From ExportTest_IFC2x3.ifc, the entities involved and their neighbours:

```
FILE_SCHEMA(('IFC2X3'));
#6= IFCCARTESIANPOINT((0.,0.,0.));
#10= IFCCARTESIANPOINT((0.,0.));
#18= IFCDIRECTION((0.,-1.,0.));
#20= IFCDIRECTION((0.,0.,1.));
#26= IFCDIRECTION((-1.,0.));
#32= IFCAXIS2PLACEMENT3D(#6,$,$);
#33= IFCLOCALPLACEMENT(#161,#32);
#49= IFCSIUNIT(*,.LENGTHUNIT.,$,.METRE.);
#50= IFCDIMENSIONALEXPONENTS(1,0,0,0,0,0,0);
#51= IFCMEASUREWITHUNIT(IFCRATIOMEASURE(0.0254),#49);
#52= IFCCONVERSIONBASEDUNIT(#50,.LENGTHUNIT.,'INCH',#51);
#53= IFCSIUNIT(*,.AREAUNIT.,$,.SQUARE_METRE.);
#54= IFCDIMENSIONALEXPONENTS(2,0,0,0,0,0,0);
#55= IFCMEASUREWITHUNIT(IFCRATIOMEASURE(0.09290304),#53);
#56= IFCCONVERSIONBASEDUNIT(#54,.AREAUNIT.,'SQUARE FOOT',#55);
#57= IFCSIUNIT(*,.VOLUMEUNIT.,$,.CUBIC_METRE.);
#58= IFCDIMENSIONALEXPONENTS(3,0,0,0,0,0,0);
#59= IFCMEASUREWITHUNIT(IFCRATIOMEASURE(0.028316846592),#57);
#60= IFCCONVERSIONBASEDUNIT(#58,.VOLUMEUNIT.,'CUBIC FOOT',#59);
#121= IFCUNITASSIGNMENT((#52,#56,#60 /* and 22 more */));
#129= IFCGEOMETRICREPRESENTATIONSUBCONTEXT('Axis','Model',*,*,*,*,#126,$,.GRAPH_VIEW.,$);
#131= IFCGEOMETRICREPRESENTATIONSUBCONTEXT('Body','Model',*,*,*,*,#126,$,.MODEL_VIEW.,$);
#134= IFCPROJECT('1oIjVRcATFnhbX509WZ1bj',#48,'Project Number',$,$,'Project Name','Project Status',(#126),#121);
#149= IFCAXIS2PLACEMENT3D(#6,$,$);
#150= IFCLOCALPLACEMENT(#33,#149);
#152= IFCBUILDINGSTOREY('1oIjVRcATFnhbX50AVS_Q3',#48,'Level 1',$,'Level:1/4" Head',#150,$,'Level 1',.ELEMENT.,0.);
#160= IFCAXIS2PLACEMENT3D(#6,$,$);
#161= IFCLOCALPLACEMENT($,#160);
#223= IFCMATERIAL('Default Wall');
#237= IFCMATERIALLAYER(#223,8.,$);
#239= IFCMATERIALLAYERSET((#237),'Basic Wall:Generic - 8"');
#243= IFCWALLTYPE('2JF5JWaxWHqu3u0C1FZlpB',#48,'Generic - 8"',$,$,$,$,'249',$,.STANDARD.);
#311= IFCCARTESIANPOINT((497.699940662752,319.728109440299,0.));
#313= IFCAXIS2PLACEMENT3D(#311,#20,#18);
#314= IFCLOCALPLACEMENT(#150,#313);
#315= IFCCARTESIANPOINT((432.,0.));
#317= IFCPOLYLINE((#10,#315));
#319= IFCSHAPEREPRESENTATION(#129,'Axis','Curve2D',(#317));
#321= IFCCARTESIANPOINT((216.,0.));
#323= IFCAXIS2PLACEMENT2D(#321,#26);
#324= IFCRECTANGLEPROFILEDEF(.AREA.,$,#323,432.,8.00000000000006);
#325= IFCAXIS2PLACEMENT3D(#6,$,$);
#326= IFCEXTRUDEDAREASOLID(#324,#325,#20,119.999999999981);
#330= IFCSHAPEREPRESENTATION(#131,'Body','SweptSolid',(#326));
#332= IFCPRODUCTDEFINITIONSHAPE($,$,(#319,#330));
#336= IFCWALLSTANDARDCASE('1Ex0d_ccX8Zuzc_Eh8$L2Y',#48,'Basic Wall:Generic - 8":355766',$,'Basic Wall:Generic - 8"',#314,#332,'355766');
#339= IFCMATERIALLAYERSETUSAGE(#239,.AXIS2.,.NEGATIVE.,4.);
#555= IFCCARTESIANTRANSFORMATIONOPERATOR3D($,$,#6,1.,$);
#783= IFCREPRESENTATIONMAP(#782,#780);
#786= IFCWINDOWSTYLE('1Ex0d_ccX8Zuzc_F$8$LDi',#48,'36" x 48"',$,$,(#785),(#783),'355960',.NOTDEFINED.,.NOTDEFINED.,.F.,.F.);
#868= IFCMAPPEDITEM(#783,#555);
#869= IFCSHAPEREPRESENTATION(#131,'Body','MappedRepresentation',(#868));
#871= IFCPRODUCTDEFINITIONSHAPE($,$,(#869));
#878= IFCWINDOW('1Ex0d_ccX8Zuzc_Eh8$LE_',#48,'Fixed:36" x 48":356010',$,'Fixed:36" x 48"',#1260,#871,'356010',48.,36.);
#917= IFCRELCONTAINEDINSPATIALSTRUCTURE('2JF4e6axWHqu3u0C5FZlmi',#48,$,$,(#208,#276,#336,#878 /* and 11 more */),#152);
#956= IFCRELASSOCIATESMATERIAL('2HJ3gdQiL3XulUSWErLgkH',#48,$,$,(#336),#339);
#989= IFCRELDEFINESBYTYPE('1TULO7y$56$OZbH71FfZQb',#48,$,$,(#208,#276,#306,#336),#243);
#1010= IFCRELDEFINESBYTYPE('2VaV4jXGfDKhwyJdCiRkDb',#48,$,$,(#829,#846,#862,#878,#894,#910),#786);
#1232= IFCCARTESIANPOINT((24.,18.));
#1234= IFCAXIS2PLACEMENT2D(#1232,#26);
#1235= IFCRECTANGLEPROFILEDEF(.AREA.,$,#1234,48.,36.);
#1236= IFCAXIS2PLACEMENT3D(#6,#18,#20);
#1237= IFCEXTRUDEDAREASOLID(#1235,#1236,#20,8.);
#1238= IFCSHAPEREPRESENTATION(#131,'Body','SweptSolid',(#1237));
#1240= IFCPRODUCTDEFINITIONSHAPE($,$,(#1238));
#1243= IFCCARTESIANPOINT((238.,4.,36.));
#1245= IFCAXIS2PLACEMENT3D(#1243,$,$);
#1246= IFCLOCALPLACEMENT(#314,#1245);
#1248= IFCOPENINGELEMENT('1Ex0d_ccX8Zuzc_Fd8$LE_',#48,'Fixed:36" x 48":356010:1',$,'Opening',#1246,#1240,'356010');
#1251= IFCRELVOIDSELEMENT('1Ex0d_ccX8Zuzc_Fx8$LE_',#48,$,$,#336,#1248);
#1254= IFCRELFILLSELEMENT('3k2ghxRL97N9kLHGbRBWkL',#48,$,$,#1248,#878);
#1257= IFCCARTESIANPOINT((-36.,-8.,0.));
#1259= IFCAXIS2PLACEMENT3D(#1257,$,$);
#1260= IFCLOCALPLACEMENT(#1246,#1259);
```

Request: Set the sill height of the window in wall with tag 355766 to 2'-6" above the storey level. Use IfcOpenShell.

```python
import numpy as np
import ifcopenshell
import ifcopenshell.api.geometry
import ifcopenshell.geom
import ifcopenshell.util.element
import ifcopenshell.util.placement
import ifcopenshell.util.shape
import ifcopenshell.util.unit

model = ifcopenshell.open("ExportTest_IFC2x3.ifc")
unit_scale = ifcopenshell.util.unit.calculate_unit_scale(model)

window = model.by_guid("1Ex0d_ccX8Zuzc_Eh8$LE_")
opening = window.FillsVoids[0].RelatingOpeningElement
storey = ifcopenshell.util.element.get_container(window, ifc_class="IfcBuildingStorey")
level = ifcopenshell.util.placement.get_local_placement(storey.ObjectPlacement)[2, 3]

# The opening's origin need not be at the sill, so measure its lowest point.
shape = ifcopenshell.geom.create_shape(ifcopenshell.geom.settings(), opening)
bottom = ifcopenshell.util.shape.get_shape_bottom_elevation(shape, shape.geometry) / unit_scale
dz = level + 30 * 0.0254 / unit_scale - bottom

shift = np.array([0.0, 0.0, dz])
# The window is placed relative to its opening, so it follows when the opening moves.
matrix = ifcopenshell.util.placement.get_local_placement(opening.ObjectPlacement)
matrix[:3, 3] += shift
ifcopenshell.api.geometry.edit_object_placement(
    model, product=opening, matrix=matrix, is_si=False, should_transform_children=True
)

print(f"moved by {dz * unit_scale:+.3f} m")

model.write("ExportTest_IFC2x3_edited.ifc")
```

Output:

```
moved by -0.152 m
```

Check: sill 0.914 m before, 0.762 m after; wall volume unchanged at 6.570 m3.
